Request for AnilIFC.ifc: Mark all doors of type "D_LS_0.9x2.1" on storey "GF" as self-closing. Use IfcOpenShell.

First a look at what the model holds.

```python
import ifcopenshell
import ifcopenshell.util.element

model = ifcopenshell.open("AnilIFC.ifc")
print(model.schema)
storey = next(s for s in model.by_type("IfcBuildingStorey") if s.Name == "GF")
doors = [e for e in ifcopenshell.util.element.get_decomposition(storey) if e.is_a("IfcDoor")]
seen = {}
for e in doors:
    element_type = ifcopenshell.util.element.get_type(e)
    key = (element_type.Name if element_type != e and element_type else None, ifcopenshell.util.element.get_pset(e, "Pset_DoorCommon", "SelfClosing"))
    seen[key] = seen.get(key, 0) + 1
for (name, value), count in sorted(seen.items(), key=str):
    print(count, "x", name, "|", value)
```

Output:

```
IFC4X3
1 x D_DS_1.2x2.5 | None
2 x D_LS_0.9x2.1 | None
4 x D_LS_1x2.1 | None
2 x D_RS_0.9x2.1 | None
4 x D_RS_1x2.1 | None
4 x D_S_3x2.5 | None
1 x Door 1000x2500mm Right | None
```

```python
import ifcopenshell
import ifcopenshell.api.pset
import ifcopenshell.util.element

model = ifcopenshell.open("AnilIFC.ifc")

storey = next(s for s in model.by_type("IfcBuildingStorey") if s.Name == "GF")
doors = [e for e in ifcopenshell.util.element.get_decomposition(storey) if e.is_a("IfcDoor")]

count = 0
for e in doors:
    element_type = ifcopenshell.util.element.get_type(e)
    if element_type in (None, e) or element_type.Name != "D_LS_0.9x2.1":
        continue
    # add_pset returns the element's existing set when there is one.
    pset = ifcopenshell.api.pset.add_pset(model, product=e, name="Pset_DoorCommon")
    ifcopenshell.api.pset.edit_pset(model, pset=pset, properties={"SelfClosing": True})
    count += 1

print(count, "doors updated")

model.write("AnilIFC_edited.ifc")
```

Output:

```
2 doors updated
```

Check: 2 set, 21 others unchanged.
